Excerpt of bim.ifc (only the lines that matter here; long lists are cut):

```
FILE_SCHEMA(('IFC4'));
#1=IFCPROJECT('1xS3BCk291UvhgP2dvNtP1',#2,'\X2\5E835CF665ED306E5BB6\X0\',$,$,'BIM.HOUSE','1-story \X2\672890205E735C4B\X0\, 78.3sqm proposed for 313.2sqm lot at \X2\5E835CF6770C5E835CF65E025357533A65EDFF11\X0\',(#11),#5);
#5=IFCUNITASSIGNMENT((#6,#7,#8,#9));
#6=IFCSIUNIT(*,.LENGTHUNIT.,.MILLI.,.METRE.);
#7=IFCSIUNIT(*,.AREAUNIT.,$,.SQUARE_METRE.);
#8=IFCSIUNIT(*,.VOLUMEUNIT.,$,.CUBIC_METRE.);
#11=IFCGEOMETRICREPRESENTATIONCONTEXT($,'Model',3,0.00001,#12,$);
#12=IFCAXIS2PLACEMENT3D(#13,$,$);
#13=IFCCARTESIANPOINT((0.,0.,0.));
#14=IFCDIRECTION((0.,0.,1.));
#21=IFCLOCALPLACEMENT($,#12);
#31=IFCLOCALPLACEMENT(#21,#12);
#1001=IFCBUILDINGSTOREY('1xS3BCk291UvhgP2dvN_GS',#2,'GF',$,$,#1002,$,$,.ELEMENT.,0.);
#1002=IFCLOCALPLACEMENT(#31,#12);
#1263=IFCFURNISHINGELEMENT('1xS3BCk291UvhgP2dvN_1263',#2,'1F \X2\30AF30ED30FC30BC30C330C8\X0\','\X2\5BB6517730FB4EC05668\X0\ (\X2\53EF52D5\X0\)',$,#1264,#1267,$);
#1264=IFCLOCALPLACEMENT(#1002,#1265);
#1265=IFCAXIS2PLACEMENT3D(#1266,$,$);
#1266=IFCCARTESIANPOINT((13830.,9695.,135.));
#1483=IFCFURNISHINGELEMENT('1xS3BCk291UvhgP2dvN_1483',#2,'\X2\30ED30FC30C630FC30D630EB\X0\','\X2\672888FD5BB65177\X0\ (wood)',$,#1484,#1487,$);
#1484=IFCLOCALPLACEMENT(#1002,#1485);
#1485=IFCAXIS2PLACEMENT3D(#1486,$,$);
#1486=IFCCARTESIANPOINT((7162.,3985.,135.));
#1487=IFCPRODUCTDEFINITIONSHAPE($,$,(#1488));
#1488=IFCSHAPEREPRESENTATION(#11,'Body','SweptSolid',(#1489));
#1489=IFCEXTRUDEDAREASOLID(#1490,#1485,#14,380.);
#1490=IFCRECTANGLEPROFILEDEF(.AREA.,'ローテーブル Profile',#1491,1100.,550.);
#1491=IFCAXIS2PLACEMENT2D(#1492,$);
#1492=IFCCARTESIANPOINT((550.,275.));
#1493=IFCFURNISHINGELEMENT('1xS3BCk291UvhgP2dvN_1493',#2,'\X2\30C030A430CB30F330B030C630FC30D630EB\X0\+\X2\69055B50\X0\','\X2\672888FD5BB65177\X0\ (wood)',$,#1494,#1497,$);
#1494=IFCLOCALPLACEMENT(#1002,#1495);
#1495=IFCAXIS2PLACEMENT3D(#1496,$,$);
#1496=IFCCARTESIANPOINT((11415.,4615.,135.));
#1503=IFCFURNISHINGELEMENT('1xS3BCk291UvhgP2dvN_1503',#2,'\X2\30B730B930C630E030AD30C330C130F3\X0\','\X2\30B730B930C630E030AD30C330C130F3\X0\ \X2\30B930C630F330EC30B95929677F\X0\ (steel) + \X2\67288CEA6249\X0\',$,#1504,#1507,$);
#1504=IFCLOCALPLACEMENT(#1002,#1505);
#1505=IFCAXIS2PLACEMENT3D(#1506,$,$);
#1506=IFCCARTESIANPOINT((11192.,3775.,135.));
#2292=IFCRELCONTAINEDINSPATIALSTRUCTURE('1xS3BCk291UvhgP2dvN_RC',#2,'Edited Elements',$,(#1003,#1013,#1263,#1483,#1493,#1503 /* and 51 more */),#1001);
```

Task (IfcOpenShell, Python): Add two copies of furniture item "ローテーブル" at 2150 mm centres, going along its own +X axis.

```python
import ifcopenshell
import ifcopenshell.api.geometry
import ifcopenshell.api.root
import ifcopenshell.util.element
import ifcopenshell.util.placement
import ifcopenshell.util.unit

model = ifcopenshell.open("bim.ifc")
unit_scale = ifcopenshell.util.unit.calculate_unit_scale(model)


def reuse_history(source, copy):
    """copy_class also copies each property set's owner history, people and application; keep the originals."""
    for rel in copy.IsDefinedBy:
        if rel.is_a("IfcRelDefinesByProperties") and (history := rel.RelatingPropertyDefinition.OwnerHistory):
            rel.RelatingPropertyDefinition.OwnerHistory = source.OwnerHistory
            ifcopenshell.util.element.remove_deep2(model, history)


source = model.by_guid("1xS3BCk291UvhgP2dvN_1483")
base = ifcopenshell.util.placement.get_local_placement(source.ObjectPlacement)
step = base[:3, 0] * 2.15 / unit_scale

for i in range(1, 3):
    copy = ifcopenshell.api.root.copy_class(model, product=source)
    copy.Representation = ifcopenshell.util.element.copy_deep(
        model, source.Representation, exclude=["IfcGeometricRepresentationContext", "IfcRepresentationMap"]
    )
    reuse_history(source, copy)
    matrix = base.copy()
    matrix[:3, 3] += i * step
    print("added at", matrix[:3, 3].round(3) + 0.0)
    ifcopenshell.api.geometry.edit_object_placement(model, product=copy, matrix=matrix, is_si=False)

model.write("bim_v2.ifc")
```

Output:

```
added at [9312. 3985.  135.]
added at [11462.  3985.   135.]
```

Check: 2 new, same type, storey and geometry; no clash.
